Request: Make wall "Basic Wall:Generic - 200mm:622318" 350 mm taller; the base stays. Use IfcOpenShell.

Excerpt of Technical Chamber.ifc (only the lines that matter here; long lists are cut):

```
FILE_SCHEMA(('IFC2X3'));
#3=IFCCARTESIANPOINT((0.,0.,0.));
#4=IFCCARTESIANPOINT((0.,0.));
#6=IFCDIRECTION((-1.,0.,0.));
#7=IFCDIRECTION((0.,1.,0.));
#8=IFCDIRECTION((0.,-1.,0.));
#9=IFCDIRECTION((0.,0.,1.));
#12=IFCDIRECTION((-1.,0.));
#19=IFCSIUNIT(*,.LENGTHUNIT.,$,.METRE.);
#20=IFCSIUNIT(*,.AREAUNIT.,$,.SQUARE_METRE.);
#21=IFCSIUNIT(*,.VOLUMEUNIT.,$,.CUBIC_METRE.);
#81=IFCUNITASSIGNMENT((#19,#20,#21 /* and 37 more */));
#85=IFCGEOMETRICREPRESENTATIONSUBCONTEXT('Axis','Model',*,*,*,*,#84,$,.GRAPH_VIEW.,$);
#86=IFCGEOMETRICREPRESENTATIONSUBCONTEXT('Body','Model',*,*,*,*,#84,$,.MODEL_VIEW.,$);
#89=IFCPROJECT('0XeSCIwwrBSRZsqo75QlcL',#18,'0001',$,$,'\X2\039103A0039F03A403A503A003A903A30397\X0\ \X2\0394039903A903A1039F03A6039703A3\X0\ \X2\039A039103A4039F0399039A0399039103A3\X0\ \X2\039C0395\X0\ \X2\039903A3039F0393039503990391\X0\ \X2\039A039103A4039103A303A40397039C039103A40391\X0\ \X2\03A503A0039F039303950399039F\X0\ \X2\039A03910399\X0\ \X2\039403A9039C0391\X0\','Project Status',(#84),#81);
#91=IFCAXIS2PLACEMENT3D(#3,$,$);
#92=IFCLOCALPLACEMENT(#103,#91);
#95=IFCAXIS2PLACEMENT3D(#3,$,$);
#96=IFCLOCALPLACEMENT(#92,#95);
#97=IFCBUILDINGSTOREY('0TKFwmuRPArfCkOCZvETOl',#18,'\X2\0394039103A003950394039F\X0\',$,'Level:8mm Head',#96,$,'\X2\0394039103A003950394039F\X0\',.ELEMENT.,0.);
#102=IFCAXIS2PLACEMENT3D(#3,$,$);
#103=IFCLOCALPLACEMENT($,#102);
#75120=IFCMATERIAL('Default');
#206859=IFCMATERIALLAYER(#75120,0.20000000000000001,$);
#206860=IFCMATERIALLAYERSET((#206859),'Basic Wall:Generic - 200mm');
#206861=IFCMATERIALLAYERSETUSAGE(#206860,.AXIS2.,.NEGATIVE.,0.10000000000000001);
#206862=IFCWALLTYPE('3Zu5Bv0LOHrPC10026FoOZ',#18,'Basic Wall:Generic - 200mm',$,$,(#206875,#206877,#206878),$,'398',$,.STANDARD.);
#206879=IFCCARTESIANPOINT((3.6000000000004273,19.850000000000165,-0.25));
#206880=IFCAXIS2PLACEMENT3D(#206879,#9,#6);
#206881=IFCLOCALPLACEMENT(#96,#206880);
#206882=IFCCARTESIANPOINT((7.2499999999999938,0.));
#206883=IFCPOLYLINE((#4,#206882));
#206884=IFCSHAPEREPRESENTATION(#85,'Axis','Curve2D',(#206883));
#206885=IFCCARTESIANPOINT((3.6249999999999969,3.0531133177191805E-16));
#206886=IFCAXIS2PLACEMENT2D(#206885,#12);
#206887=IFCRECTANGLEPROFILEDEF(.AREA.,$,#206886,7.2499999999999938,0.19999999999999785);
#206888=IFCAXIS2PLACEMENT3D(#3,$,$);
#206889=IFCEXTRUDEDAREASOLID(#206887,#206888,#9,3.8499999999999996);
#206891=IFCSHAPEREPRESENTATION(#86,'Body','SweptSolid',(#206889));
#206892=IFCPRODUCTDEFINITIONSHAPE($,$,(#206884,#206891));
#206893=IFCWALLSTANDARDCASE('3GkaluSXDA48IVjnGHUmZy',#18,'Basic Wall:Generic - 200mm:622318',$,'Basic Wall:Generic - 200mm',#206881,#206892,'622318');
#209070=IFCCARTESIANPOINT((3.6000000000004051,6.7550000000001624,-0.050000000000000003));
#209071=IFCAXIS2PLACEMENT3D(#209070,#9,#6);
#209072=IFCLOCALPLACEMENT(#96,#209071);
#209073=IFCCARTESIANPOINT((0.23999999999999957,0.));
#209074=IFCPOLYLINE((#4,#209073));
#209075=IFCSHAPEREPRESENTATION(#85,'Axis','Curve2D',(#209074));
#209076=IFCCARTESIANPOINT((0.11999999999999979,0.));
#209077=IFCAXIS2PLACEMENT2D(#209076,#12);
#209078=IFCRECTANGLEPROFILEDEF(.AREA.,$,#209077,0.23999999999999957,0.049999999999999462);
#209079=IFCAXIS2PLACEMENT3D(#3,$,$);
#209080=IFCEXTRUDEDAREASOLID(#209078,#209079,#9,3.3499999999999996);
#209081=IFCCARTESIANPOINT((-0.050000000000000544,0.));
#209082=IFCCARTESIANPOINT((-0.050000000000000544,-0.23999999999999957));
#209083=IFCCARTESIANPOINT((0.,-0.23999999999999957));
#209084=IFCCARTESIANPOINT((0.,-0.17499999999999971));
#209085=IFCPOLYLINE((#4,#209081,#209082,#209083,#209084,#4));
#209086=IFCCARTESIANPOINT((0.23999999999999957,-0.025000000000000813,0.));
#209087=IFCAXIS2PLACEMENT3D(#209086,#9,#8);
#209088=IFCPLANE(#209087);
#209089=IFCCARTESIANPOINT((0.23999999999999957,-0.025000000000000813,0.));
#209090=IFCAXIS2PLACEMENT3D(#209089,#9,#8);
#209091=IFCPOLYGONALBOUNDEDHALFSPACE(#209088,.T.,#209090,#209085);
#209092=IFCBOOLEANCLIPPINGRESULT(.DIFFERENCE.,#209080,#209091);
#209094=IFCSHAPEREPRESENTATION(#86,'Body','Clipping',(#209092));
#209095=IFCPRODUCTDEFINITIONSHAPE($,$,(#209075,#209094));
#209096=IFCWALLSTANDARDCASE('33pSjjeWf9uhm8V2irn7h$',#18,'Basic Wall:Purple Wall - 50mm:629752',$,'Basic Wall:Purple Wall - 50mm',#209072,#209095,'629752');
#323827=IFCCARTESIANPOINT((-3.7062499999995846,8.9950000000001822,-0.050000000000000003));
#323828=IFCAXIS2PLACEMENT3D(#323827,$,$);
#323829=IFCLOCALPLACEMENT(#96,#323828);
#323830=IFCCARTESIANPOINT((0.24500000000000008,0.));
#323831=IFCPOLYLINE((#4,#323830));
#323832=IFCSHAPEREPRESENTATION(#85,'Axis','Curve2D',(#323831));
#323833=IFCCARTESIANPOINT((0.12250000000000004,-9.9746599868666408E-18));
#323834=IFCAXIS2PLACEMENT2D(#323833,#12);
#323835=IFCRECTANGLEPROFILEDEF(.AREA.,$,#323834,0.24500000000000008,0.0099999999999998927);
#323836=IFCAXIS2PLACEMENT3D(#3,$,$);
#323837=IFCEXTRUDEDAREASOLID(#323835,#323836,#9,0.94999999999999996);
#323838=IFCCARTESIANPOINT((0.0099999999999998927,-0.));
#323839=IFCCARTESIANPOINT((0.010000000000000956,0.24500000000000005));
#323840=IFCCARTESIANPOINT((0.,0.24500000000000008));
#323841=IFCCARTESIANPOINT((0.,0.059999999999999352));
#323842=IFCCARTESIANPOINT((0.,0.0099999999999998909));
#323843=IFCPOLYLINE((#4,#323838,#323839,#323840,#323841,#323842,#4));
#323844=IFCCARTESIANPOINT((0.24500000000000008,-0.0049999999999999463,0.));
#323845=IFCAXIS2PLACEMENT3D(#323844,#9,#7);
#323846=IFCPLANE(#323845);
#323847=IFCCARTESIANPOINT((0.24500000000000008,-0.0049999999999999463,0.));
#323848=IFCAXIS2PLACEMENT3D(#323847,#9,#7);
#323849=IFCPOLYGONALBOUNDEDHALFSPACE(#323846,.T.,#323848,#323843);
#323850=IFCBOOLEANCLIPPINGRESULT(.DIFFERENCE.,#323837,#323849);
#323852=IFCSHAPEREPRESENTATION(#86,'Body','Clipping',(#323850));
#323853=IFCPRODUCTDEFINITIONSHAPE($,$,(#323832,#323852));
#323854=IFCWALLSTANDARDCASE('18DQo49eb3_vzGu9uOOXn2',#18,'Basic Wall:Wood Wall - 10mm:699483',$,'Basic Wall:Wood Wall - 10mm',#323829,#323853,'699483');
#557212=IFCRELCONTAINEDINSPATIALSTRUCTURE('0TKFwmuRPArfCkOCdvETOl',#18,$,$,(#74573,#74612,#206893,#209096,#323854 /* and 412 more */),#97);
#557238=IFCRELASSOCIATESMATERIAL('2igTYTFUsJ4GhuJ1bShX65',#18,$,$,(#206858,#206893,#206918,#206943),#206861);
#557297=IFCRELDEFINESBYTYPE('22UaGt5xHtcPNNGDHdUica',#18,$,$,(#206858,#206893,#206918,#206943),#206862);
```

```python
import ifcopenshell
import ifcopenshell.geom
import ifcopenshell.util.representation
import ifcopenshell.util.shape

model = ifcopenshell.open("Technical Chamber.ifc")
settings = ifcopenshell.geom.settings()


def volume(element):
    """Net volume in cubic metres, openings subtracted."""
    shape = ifcopenshell.geom.create_shape(settings, element)
    return ifcopenshell.util.shape.get_volume(shape.geometry)


wall = model.by_guid("3GkaluSXDA48IVjnGHUmZy")
before = volume(wall)

body = ifcopenshell.util.representation.get_representation(wall, "Model", "Body")
solid = body.Items[0]
old_height = solid.Depth
solid.Depth += 0.35
after = volume(wall)

print(f"height {old_height:g} -> {solid.Depth:g}, volume {before:.3f} -> {after:.3f} m3")

model.write("Technical Chamber-out.ifc")
```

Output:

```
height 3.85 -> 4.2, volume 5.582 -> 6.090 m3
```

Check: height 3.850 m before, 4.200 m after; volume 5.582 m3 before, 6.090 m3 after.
